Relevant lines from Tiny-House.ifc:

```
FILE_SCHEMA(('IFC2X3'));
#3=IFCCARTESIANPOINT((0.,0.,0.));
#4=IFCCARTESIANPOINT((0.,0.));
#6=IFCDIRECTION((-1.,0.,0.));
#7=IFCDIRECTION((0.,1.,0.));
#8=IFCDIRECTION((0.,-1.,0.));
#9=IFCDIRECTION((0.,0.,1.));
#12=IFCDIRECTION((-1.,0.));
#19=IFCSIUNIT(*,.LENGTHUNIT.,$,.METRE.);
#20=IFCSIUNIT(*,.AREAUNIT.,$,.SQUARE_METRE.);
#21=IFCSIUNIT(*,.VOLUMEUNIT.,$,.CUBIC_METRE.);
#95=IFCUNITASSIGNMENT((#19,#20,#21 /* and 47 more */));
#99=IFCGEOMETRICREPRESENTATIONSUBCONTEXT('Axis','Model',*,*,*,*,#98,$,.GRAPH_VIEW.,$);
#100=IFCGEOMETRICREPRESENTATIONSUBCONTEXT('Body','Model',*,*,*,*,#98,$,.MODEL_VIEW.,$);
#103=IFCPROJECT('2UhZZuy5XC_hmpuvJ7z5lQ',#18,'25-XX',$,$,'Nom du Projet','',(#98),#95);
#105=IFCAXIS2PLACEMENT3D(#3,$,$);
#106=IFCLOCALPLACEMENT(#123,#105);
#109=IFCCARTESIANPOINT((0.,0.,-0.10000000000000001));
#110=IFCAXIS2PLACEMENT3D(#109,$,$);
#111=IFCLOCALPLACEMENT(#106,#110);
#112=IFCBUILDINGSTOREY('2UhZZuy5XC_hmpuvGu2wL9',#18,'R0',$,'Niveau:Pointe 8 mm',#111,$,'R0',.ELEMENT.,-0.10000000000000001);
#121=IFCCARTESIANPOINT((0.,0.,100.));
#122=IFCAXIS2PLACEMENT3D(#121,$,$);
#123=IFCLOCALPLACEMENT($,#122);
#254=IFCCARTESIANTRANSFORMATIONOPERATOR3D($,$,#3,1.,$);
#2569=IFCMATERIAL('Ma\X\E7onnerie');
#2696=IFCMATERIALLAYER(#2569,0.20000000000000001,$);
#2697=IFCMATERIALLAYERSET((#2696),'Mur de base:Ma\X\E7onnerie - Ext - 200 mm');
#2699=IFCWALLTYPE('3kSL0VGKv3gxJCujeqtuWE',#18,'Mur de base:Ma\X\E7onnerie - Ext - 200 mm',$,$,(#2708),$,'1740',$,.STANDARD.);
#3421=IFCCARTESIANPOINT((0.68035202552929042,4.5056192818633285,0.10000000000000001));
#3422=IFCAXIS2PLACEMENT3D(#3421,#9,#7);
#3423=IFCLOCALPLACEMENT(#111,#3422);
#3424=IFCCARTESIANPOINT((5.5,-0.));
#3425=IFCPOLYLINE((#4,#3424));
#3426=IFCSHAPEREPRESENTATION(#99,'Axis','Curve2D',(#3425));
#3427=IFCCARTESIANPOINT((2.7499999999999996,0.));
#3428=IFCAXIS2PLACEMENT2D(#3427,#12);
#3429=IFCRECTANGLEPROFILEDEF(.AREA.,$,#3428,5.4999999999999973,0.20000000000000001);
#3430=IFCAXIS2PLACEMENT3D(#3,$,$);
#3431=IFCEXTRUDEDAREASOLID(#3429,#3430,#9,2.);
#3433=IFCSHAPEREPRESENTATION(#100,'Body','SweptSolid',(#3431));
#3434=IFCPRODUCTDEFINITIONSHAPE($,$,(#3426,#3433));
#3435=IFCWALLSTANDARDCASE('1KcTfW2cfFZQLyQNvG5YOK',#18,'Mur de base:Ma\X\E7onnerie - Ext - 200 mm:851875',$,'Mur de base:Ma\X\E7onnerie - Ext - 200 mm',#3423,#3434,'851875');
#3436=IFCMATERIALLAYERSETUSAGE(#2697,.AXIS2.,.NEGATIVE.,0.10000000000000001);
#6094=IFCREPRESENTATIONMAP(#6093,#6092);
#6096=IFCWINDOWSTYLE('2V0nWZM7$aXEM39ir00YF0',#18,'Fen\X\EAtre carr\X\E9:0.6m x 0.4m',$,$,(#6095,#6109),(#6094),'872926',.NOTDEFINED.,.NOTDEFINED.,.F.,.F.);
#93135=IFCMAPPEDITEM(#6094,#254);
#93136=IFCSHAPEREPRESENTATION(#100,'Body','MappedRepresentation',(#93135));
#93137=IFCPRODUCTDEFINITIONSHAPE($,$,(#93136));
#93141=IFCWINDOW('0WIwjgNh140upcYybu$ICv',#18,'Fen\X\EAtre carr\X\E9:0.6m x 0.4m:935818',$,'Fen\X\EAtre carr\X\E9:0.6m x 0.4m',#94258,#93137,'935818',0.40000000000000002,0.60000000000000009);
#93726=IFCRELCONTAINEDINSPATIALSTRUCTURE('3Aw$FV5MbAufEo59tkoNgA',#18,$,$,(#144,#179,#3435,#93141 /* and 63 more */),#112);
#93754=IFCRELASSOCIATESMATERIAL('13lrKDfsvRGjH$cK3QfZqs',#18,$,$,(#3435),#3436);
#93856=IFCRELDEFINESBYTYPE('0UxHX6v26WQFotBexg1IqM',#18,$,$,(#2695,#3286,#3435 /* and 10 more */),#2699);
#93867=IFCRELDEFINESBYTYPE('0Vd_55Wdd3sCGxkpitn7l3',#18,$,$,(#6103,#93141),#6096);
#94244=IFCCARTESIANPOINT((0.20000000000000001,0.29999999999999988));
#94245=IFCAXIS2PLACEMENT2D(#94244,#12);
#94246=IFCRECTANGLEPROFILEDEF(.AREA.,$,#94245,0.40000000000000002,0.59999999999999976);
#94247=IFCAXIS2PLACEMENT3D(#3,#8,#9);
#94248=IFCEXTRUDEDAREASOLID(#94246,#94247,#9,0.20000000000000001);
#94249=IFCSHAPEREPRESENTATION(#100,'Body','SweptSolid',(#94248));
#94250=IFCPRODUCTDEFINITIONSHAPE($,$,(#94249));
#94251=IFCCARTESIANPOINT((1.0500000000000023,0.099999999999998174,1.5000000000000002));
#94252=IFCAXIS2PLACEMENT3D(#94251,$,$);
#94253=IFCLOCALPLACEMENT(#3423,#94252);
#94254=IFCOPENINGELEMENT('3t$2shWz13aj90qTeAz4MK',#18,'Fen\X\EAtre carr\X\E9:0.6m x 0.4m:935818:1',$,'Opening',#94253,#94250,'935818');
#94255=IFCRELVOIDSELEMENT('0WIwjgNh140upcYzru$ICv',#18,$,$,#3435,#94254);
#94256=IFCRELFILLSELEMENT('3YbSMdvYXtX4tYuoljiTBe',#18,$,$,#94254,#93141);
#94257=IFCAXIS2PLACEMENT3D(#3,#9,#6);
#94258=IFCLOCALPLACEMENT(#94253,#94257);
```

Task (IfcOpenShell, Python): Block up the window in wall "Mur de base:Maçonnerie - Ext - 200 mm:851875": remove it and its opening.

```python
import ifcopenshell
import ifcopenshell.api.feature
import ifcopenshell.api.root
import ifcopenshell.geom
import ifcopenshell.util.shape

model = ifcopenshell.open("Tiny-House.ifc")
settings = ifcopenshell.geom.settings()


def volume(element):
    """Net volume in cubic metres, openings subtracted."""
    shape = ifcopenshell.geom.create_shape(settings, element)
    return ifcopenshell.util.shape.get_volume(shape.geometry)


window = model.by_guid("0WIwjgNh140upcYybu$ICv")
opening = window.FillsVoids[0].RelatingOpeningElement
wall = opening.VoidsElements[0].RelatingBuildingElement
before = volume(wall)

ifcopenshell.api.root.remove_product(model, product=window)
ifcopenshell.api.feature.remove_feature(model, feature=opening)

after = volume(wall)

print(f"wall volume {before:.3f} -> {after:.3f} m3")

model.write("Tiny-House_updated.ifc")
```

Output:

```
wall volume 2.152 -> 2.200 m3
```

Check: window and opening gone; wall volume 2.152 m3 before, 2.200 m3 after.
